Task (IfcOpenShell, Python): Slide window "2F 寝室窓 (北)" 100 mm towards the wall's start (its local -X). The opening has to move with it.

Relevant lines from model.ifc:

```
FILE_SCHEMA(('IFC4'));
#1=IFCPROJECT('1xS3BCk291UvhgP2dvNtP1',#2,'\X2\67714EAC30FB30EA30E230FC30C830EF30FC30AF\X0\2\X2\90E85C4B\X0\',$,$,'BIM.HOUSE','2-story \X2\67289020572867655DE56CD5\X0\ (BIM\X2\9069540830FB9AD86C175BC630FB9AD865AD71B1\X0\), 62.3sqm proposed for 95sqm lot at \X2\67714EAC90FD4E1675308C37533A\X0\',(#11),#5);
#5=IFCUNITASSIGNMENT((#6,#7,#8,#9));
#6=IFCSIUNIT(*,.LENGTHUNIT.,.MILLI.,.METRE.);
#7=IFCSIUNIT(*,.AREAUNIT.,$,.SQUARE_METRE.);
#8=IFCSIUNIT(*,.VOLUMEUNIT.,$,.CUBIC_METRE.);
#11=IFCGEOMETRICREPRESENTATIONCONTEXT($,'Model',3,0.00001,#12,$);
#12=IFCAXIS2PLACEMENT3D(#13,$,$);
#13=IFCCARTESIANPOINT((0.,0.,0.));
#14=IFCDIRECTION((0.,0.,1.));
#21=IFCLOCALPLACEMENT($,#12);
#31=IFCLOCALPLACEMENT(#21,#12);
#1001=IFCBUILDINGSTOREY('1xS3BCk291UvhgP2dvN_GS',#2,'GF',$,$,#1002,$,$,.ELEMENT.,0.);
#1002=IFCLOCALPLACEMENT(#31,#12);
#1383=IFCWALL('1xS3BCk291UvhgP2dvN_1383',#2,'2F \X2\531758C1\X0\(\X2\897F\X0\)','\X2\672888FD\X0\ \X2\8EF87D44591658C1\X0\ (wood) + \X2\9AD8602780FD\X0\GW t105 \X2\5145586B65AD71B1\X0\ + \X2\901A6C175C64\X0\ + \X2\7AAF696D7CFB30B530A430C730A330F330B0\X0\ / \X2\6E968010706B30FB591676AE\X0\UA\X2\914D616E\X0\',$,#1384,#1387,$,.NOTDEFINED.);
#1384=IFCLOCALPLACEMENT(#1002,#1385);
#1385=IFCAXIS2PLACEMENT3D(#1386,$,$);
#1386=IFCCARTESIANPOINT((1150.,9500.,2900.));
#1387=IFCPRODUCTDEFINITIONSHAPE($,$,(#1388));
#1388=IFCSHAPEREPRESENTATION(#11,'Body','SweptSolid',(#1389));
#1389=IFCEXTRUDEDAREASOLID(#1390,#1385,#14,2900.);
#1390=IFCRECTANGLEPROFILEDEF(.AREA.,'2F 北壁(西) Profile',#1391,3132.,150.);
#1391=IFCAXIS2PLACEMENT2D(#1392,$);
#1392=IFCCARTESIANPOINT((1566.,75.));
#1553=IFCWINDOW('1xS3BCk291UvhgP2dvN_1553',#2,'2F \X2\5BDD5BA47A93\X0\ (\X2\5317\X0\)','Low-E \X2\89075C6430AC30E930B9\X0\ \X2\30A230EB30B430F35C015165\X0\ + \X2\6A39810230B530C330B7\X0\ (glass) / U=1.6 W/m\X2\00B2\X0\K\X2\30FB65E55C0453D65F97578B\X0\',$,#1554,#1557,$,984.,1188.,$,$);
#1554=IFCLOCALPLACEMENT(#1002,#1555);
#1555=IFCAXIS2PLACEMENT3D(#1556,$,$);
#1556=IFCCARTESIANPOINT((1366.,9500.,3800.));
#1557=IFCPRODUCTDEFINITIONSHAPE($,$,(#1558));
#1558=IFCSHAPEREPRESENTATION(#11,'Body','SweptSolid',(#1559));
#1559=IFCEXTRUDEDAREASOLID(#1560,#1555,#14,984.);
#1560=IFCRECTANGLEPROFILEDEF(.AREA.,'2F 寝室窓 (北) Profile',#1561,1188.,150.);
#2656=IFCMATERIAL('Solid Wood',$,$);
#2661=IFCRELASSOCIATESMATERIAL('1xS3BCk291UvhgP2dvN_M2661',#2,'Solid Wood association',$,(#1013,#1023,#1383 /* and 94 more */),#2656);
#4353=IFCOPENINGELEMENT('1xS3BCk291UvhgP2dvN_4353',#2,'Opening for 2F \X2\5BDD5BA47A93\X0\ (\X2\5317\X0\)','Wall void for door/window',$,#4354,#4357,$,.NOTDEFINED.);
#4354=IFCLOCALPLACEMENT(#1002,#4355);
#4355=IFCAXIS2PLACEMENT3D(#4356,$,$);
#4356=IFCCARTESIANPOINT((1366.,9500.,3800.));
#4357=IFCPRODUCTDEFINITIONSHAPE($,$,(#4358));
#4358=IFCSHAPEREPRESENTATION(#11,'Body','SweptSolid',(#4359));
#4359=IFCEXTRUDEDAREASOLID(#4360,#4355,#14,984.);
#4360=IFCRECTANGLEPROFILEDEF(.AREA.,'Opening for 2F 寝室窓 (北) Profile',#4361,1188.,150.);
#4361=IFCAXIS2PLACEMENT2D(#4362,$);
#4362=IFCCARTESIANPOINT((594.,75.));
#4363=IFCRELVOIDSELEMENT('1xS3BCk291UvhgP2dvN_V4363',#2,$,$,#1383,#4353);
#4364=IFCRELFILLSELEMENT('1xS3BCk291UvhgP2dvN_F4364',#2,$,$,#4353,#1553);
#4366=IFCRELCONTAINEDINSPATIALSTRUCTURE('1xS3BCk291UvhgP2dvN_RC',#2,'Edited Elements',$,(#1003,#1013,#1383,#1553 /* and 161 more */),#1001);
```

```python
import ifcopenshell
import ifcopenshell.api.geometry
import ifcopenshell.util.placement

model = ifcopenshell.open("model.ifc")

window = model.by_guid("1xS3BCk291UvhgP2dvN_1553")
opening = window.FillsVoids[0].RelatingOpeningElement
wall = opening.VoidsElements[0].RelatingBuildingElement

wall_matrix = ifcopenshell.util.placement.get_local_placement(wall.ObjectPlacement)
shift = wall_matrix[:3, 0] * -100.0
before = ifcopenshell.util.placement.get_local_placement(window.ObjectPlacement)[:3, 3].copy()

# The window is not placed relative to its opening, so move both.
for product in (opening, window):
    matrix = ifcopenshell.util.placement.get_local_placement(product.ObjectPlacement)
    matrix[:3, 3] += shift
    ifcopenshell.api.geometry.edit_object_placement(model, product=product, matrix=matrix, is_si=False)

after = ifcopenshell.util.placement.get_local_placement(window.ObjectPlacement)[:3, 3]
print("window moved by", (after - before).round(3) + 0.0)

model.write("model_updated.ifc")
```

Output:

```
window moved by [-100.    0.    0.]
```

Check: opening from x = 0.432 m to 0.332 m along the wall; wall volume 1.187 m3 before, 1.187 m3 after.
